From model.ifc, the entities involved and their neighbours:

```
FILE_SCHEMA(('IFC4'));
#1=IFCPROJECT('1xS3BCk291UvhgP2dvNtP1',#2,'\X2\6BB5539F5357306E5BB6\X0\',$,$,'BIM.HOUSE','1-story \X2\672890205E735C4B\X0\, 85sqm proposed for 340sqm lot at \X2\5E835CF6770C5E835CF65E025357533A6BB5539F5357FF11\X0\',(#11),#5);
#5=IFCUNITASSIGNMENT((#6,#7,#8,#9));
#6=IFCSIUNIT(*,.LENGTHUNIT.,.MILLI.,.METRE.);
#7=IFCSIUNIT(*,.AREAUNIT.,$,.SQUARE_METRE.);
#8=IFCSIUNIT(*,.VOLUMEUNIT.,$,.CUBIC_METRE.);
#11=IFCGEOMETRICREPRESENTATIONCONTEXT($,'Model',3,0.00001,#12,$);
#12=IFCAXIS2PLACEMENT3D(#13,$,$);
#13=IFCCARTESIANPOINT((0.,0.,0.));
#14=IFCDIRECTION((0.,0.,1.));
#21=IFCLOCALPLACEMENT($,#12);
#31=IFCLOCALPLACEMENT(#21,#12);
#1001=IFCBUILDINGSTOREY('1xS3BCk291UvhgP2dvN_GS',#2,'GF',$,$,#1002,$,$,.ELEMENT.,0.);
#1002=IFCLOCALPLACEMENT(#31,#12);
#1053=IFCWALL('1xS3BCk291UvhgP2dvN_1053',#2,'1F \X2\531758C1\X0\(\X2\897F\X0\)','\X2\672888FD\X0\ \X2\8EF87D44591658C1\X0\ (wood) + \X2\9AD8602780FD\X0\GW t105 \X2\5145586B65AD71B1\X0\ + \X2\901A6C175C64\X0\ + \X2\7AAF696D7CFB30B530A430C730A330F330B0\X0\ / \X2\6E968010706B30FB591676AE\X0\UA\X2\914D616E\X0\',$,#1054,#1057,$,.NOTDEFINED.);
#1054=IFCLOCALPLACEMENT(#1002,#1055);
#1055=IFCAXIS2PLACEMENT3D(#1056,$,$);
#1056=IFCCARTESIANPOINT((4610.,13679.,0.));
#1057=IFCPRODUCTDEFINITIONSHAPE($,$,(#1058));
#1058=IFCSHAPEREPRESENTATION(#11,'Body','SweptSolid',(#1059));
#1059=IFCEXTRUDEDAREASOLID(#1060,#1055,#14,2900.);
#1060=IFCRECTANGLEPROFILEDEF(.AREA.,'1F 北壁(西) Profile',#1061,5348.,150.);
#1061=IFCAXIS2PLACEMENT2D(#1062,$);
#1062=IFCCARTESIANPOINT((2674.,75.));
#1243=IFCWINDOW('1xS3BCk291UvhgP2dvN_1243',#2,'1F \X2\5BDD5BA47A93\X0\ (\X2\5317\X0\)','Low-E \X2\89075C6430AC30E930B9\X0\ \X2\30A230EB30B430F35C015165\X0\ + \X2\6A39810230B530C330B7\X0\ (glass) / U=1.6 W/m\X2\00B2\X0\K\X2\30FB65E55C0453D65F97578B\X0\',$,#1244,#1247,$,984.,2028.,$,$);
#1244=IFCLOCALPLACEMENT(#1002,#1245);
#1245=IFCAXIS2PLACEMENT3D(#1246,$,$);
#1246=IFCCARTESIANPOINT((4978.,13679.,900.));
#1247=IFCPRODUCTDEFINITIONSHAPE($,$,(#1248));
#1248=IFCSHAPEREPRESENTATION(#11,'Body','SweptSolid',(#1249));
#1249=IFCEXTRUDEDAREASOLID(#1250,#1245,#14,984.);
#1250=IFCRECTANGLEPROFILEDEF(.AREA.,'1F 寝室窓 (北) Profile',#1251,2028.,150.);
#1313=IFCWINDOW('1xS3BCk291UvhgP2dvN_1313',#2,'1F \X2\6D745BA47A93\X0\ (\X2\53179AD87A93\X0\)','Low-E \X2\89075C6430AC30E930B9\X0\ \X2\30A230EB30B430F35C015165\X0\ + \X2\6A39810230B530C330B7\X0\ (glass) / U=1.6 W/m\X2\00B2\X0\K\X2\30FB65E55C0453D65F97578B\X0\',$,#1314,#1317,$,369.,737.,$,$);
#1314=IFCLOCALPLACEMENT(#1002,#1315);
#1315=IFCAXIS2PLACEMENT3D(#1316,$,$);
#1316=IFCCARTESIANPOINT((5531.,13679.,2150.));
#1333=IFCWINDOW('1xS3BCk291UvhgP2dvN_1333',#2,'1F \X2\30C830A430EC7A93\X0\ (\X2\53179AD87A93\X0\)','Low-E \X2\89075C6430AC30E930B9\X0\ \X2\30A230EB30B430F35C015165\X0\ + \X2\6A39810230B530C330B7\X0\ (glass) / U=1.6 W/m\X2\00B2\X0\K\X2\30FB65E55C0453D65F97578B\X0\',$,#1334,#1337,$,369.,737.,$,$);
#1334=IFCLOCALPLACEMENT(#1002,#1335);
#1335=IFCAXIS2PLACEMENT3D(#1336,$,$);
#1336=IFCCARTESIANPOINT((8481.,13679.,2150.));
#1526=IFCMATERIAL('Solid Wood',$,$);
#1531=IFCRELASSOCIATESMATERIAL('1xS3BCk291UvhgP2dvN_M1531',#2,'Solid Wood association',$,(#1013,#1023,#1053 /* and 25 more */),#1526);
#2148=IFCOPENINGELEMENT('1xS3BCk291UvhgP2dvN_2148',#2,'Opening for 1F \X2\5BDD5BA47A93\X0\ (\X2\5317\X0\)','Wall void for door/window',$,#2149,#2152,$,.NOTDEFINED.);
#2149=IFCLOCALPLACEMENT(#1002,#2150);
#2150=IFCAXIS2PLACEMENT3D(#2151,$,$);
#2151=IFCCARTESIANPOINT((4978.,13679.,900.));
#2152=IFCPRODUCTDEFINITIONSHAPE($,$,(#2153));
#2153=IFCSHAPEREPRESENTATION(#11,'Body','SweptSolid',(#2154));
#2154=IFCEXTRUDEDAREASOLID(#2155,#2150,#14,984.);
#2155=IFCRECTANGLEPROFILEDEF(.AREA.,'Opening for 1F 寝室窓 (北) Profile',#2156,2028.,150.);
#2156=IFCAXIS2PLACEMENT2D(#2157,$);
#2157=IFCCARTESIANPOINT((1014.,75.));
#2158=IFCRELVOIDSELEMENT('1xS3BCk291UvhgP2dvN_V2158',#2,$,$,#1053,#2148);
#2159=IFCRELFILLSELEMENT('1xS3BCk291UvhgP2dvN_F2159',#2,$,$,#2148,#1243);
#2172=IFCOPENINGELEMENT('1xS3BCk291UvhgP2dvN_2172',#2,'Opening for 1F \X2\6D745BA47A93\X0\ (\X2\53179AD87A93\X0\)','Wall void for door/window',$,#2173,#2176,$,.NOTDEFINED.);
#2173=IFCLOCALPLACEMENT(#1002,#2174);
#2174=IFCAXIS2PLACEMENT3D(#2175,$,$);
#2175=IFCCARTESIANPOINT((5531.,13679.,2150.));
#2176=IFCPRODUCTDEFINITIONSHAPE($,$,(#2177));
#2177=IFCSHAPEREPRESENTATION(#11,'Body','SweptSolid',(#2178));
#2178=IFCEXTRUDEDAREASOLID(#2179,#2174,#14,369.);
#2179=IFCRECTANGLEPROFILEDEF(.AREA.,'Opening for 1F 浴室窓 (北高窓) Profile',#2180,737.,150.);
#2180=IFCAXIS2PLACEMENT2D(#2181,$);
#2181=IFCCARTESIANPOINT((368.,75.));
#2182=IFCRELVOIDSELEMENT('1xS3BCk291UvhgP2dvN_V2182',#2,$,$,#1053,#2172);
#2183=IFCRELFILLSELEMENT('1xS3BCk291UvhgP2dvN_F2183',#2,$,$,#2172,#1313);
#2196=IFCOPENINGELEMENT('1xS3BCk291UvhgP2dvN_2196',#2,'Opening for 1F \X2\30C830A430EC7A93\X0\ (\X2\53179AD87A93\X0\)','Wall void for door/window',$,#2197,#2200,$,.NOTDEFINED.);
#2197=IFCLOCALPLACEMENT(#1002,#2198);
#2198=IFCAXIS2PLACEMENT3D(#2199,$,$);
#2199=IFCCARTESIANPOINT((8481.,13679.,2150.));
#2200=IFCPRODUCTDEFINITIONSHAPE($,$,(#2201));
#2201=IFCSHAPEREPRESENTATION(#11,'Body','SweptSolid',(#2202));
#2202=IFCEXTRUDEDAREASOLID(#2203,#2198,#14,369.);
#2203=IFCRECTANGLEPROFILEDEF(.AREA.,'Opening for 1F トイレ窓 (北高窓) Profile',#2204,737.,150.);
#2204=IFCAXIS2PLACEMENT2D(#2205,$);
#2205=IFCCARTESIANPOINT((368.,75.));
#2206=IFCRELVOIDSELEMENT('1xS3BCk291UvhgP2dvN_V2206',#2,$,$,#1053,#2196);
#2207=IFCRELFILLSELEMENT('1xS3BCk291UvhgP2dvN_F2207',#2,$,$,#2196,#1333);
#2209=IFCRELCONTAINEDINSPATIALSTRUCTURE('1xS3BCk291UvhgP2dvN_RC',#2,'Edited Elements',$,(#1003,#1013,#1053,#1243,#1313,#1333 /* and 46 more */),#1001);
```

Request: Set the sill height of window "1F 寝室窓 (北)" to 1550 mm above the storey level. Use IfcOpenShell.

```python
import numpy as np
import ifcopenshell
import ifcopenshell.api.geometry
import ifcopenshell.geom
import ifcopenshell.util.element
import ifcopenshell.util.placement
import ifcopenshell.util.shape
import ifcopenshell.util.unit

model = ifcopenshell.open("model.ifc")
unit_scale = ifcopenshell.util.unit.calculate_unit_scale(model)

window = model.by_guid("1xS3BCk291UvhgP2dvN_1243")
opening = window.FillsVoids[0].RelatingOpeningElement
storey = ifcopenshell.util.element.get_container(window, ifc_class="IfcBuildingStorey")
level = ifcopenshell.util.placement.get_local_placement(storey.ObjectPlacement)[2, 3]

# The opening's origin need not be at the sill, so measure its lowest point.
shape = ifcopenshell.geom.create_shape(ifcopenshell.geom.settings(), opening)
bottom = ifcopenshell.util.shape.get_shape_bottom_elevation(shape, shape.geometry) / unit_scale
dz = level + 1.55 / unit_scale - bottom

shift = np.array([0.0, 0.0, dz])
# The window is not placed relative to its opening, so move both.
for product in (opening, window):
    matrix = ifcopenshell.util.placement.get_local_placement(product.ObjectPlacement)
    matrix[:3, 3] += shift
    ifcopenshell.api.geometry.edit_object_placement(model, product=product, matrix=matrix, is_si=False)

print(f"moved by {dz * unit_scale:+.3f} m")

model.write("model_edited.ifc")
```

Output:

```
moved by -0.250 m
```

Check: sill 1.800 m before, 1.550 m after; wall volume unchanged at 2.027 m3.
